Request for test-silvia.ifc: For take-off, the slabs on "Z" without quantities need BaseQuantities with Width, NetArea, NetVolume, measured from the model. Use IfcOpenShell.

First a look at what the model holds.

```python
import ifcopenshell
import ifcopenshell.util.element
import ifcopenshell.util.unit

model = ifcopenshell.open("test-silvia.ifc")
print(model.schema)
for unit_type in ("LENGTHUNIT", "AREAUNIT", "VOLUMEUNIT"):
    print(unit_type, ifcopenshell.util.unit.calculate_unit_scale(model, unit_type))
storey = next(s for s in model.by_type("IfcBuildingStorey") if s.Name == "Z")
slabs = [e for e in ifcopenshell.util.element.get_decomposition(storey) if e.is_a("IfcSlab")]
for e in sorted(slabs, key=lambda e: e.id()):
    print(e.id(), e.is_a(), e.Name, list(ifcopenshell.util.element.get_psets(e, qtos_only=True)), sep=" | ")
```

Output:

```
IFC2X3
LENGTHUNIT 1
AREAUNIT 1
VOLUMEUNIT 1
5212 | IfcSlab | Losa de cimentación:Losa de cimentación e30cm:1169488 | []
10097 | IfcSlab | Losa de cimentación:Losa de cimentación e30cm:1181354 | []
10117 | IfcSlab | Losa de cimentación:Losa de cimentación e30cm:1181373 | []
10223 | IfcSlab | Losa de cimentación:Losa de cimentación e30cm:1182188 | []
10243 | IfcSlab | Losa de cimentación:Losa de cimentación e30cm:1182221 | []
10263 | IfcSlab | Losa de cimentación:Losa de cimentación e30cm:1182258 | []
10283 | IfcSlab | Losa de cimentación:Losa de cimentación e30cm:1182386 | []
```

```python
import ifcopenshell
import ifcopenshell.api.pset
import ifcopenshell.geom
import ifcopenshell.util.element
import ifcopenshell.util.shape
import ifcopenshell.util.unit

model = ifcopenshell.open("test-silvia.ifc")
unit_scale = ifcopenshell.util.unit.calculate_unit_scale(model)
area_scale = ifcopenshell.util.unit.calculate_unit_scale(model, "AREAUNIT")
volume_scale = ifcopenshell.util.unit.calculate_unit_scale(model, "VOLUMEUNIT")
settings = ifcopenshell.geom.settings()

storey = next(s for s in model.by_type("IfcBuildingStorey") if s.Name == "Z")
slabs = [e for e in ifcopenshell.util.element.get_decomposition(storey) if e.is_a("IfcSlab")]

for e in sorted(slabs, key=lambda e: e.id()):
    if ifcopenshell.util.element.get_psets(e, qtos_only=True, should_inherit=False):
        continue
    # Geometry comes back in metres, in the element's own axes.
    shape = ifcopenshell.geom.create_shape(settings, e)
    values = {
        "Width": ifcopenshell.util.shape.get_z(shape.geometry) / unit_scale,
        "NetArea": ifcopenshell.util.shape.get_footprint_area(shape.geometry) / area_scale,
        "NetVolume": ifcopenshell.util.shape.get_volume(shape.geometry) / volume_scale,
    }
    qto = ifcopenshell.api.pset.add_qto(model, product=e, name="BaseQuantities")
    ifcopenshell.api.pset.edit_qto(model, qto=qto, properties=values)
    print(e.id(), {k: round(v, 3) for k, v in values.items()})

model.write("test-silvia_edited.ifc")
```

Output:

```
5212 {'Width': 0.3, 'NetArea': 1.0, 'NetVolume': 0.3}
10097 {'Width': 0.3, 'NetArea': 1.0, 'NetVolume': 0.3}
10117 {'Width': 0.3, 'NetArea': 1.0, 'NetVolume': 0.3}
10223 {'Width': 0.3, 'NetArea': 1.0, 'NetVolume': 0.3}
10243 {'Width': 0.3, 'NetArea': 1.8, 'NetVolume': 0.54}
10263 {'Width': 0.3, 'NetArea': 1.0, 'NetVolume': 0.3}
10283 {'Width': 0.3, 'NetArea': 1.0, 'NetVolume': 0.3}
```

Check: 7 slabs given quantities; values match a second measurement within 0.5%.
